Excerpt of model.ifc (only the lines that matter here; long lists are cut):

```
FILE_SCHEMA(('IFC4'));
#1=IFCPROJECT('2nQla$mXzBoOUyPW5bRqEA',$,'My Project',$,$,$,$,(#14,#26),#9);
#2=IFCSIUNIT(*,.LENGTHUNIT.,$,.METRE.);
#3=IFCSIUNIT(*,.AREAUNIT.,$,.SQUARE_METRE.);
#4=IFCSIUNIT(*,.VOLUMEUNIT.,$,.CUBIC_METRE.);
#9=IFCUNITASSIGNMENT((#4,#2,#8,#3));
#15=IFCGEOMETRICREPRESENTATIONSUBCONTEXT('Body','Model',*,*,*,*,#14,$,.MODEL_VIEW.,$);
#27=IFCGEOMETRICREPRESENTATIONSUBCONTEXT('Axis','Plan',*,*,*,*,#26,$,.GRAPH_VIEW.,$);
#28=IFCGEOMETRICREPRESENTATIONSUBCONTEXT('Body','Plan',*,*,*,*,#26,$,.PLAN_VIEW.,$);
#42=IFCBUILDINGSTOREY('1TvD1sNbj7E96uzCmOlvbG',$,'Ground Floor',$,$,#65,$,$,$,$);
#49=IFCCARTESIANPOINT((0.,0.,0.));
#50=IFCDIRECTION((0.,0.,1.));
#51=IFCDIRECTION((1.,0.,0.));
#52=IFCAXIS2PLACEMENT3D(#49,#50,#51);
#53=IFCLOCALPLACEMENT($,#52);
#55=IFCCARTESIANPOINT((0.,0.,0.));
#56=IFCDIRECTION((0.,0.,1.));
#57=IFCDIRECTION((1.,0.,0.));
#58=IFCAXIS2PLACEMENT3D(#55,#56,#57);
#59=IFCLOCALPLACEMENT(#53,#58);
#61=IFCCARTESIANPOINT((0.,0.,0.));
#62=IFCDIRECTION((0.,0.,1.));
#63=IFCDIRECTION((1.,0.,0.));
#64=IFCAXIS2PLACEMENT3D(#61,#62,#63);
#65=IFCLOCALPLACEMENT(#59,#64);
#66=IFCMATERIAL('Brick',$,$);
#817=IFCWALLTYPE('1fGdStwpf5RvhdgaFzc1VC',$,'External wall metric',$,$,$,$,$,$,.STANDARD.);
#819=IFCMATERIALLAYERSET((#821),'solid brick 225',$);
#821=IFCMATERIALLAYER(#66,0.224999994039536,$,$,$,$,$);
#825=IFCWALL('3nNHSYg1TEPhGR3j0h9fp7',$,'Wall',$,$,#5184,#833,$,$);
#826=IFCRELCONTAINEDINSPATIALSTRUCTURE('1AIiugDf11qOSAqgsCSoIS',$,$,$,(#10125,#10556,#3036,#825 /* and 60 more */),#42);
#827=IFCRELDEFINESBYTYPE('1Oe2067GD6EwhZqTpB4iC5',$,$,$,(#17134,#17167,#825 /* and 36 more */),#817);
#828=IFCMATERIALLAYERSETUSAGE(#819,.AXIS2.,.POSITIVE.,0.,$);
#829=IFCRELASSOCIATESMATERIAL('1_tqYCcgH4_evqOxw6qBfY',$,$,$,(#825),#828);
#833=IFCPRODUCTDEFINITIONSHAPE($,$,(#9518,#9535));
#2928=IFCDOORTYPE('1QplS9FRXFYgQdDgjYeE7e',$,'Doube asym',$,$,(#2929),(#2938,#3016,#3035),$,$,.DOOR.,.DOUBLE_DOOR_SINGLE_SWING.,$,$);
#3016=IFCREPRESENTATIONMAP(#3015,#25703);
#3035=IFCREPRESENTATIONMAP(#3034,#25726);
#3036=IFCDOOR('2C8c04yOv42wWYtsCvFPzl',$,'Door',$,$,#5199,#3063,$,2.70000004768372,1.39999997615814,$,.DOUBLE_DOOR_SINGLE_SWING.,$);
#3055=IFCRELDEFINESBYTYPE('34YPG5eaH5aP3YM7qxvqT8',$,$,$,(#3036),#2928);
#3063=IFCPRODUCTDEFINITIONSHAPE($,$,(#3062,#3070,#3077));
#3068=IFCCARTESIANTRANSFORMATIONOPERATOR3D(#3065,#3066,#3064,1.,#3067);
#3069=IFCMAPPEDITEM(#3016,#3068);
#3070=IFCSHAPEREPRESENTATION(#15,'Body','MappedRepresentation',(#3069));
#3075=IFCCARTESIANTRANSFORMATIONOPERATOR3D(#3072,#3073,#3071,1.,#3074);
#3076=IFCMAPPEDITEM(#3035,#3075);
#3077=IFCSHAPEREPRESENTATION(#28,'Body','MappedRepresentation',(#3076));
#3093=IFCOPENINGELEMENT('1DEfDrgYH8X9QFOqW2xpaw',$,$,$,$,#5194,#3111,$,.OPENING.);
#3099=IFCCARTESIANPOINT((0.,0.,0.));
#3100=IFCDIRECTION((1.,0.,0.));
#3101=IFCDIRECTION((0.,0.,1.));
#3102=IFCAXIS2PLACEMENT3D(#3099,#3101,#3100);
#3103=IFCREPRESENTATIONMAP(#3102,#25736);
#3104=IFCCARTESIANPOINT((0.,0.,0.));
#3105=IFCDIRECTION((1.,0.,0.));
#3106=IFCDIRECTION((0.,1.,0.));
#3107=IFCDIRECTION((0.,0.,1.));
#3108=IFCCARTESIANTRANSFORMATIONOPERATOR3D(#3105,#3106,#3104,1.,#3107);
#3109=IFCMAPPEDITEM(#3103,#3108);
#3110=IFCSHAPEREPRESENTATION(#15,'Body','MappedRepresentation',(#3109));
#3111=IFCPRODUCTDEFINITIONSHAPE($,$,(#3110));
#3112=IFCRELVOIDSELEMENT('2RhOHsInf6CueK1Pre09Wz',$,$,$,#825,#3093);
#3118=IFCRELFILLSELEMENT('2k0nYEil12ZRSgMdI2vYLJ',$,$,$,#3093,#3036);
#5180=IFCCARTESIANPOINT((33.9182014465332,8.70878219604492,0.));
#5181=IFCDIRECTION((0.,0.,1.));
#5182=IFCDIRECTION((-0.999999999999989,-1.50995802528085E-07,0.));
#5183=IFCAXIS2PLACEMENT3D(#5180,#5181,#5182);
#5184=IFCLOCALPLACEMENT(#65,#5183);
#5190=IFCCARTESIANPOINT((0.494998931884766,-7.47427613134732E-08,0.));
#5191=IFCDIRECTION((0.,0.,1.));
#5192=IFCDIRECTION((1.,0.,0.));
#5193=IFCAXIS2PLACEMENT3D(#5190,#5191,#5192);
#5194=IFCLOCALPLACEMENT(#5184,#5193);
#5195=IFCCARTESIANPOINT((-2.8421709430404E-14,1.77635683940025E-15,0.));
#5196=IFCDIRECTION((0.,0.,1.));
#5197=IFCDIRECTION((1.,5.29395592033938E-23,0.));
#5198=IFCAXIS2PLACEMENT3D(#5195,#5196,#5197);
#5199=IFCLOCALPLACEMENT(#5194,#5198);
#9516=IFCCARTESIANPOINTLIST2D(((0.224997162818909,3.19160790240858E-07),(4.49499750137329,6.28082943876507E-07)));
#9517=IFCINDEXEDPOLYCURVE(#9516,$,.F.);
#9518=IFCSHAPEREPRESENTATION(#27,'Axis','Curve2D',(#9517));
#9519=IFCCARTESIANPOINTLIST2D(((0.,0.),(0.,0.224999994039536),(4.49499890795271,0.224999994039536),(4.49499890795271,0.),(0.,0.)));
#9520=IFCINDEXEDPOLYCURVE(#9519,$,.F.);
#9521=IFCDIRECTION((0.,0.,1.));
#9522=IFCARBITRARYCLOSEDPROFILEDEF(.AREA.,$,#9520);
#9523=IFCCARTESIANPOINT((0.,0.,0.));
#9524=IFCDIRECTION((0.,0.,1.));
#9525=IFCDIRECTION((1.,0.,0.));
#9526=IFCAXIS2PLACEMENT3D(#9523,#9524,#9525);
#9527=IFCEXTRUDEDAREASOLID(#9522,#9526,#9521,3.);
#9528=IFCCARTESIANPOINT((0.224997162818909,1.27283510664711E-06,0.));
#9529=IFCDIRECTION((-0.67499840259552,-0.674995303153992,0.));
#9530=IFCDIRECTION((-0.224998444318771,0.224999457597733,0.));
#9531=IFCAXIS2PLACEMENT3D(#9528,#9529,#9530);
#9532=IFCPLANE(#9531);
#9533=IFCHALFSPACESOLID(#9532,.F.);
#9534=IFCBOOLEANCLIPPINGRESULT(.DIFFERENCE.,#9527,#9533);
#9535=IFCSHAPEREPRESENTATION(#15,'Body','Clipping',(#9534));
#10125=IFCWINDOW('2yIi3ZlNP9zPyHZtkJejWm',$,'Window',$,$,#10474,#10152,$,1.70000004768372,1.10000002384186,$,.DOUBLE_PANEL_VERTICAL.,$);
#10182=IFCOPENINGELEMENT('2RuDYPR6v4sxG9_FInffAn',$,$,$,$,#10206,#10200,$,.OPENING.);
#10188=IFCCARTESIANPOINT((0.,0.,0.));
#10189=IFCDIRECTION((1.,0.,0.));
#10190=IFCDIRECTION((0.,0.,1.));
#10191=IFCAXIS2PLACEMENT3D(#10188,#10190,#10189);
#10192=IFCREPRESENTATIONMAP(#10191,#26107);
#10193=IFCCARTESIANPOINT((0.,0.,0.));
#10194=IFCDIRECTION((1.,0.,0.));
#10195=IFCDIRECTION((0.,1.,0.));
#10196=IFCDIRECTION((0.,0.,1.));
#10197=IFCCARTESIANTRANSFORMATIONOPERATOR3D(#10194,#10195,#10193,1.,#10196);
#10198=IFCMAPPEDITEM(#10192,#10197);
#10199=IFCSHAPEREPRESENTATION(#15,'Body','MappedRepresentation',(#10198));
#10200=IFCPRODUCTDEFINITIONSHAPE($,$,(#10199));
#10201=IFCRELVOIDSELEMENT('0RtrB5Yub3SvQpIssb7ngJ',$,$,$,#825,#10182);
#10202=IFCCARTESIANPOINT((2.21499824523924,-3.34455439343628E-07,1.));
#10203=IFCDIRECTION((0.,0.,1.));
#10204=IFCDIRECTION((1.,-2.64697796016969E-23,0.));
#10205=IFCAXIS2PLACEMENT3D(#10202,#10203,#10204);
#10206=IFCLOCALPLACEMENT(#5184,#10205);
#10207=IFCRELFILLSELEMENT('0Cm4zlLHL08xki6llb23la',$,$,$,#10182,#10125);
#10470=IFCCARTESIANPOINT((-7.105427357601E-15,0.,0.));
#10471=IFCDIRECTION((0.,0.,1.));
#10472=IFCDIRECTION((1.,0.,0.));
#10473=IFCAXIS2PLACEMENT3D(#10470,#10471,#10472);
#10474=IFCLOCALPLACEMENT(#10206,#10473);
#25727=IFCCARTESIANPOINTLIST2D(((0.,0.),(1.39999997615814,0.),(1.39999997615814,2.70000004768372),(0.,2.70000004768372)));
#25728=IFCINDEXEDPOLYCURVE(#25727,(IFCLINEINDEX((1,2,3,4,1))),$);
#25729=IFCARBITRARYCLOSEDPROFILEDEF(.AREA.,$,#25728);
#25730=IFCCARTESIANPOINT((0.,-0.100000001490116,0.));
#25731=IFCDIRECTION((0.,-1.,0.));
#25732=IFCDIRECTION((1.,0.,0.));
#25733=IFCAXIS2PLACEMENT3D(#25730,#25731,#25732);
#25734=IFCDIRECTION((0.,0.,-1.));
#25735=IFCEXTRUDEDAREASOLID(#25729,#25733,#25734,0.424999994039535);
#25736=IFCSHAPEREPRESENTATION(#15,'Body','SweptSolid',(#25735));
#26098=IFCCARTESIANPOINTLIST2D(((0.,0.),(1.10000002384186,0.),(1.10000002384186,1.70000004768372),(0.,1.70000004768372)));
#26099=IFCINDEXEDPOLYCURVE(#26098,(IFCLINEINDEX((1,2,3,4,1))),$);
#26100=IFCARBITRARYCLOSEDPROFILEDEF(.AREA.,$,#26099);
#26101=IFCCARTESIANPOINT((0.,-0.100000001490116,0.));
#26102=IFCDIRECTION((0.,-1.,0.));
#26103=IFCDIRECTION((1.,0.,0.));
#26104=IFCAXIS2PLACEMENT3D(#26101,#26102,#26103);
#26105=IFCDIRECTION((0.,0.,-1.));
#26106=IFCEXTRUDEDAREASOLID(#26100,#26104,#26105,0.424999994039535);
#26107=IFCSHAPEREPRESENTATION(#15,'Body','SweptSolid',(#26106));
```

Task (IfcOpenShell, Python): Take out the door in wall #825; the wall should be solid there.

```python
import ifcopenshell
import ifcopenshell.api.feature
import ifcopenshell.api.root
import ifcopenshell.geom
import ifcopenshell.util.shape

model = ifcopenshell.open("model.ifc")
settings = ifcopenshell.geom.settings()


def volume(element):
    """Net volume in cubic metres, openings subtracted."""
    shape = ifcopenshell.geom.create_shape(settings, element)
    return ifcopenshell.util.shape.get_volume(shape.geometry)


door = model.by_guid("2C8c04yOv42wWYtsCvFPzl")
opening = door.FillsVoids[0].RelatingOpeningElement
wall = opening.VoidsElements[0].RelatingBuildingElement
before = volume(wall)

ifcopenshell.api.root.remove_product(model, product=door)
ifcopenshell.api.feature.remove_feature(model, feature=opening)

after = volume(wall)

print(f"wall volume {before:.3f} -> {after:.3f} m3")

model.write("model_edited.ifc")
```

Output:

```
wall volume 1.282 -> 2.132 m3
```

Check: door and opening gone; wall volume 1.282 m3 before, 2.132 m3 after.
